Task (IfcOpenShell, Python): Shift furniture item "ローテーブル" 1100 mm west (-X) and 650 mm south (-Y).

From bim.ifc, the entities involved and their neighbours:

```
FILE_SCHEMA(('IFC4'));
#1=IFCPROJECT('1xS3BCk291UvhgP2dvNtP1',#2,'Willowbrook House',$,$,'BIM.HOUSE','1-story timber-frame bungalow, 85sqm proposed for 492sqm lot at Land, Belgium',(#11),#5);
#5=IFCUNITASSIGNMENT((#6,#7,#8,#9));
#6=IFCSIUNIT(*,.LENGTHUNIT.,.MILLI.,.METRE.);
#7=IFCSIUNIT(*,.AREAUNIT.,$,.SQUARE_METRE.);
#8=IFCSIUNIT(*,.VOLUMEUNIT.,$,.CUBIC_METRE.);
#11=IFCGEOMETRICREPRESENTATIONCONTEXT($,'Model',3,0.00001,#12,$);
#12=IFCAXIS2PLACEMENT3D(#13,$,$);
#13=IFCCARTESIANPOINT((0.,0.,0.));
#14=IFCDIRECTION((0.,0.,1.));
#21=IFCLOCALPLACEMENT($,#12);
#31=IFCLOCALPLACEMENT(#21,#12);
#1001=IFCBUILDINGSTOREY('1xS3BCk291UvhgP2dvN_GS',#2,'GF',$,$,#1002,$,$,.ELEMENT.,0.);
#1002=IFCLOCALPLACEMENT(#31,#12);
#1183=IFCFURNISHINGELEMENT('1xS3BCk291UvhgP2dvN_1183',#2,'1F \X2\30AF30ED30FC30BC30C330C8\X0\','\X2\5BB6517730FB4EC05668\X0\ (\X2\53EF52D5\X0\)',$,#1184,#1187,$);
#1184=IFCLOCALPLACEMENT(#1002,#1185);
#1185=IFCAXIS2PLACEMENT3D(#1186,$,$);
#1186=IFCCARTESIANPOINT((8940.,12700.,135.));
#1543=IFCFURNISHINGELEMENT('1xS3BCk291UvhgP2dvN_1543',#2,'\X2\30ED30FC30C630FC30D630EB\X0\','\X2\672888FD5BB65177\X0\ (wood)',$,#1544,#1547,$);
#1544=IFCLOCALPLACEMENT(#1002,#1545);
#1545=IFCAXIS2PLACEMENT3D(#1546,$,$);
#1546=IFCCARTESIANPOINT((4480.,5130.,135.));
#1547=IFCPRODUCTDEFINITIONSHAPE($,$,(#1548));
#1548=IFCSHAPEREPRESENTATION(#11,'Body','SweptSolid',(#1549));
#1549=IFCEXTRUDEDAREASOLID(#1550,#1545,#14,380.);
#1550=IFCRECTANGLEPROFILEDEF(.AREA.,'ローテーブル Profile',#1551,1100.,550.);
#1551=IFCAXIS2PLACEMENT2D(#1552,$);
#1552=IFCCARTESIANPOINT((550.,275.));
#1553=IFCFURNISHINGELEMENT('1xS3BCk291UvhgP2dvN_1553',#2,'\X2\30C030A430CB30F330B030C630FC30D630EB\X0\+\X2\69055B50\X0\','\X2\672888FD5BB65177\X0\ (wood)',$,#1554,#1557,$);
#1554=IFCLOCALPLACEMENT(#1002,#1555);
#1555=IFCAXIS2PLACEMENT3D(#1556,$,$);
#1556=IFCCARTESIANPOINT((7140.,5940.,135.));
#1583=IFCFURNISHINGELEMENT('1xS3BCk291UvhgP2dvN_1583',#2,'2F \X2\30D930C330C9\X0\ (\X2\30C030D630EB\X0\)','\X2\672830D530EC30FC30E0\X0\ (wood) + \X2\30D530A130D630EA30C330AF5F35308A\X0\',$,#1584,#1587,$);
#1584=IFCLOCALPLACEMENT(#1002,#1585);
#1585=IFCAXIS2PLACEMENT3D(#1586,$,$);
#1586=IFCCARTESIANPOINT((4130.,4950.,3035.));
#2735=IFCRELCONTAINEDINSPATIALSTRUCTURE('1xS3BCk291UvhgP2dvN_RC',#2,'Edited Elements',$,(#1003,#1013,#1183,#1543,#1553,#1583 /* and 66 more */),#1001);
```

```python
import ifcopenshell
import ifcopenshell.api.geometry
import ifcopenshell.util.placement
import ifcopenshell.util.unit

model = ifcopenshell.open("bim.ifc")
unit_scale = ifcopenshell.util.unit.calculate_unit_scale(model)

item = model.by_id(1543)
matrix = ifcopenshell.util.placement.get_local_placement(item.ObjectPlacement)
matrix[0, 3] -= 1.1 / unit_scale
matrix[1, 3] -= 0.65 / unit_scale
ifcopenshell.api.geometry.edit_object_placement(model, product=item, matrix=matrix, is_si=False)

print(ifcopenshell.util.placement.get_local_placement(item.ObjectPlacement).round(3) + 0.0)

model.write("bim_rev.ifc")
```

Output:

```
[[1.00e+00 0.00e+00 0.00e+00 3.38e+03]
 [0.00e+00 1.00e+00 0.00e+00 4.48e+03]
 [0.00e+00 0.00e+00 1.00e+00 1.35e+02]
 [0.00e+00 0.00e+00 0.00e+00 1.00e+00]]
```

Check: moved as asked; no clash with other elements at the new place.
